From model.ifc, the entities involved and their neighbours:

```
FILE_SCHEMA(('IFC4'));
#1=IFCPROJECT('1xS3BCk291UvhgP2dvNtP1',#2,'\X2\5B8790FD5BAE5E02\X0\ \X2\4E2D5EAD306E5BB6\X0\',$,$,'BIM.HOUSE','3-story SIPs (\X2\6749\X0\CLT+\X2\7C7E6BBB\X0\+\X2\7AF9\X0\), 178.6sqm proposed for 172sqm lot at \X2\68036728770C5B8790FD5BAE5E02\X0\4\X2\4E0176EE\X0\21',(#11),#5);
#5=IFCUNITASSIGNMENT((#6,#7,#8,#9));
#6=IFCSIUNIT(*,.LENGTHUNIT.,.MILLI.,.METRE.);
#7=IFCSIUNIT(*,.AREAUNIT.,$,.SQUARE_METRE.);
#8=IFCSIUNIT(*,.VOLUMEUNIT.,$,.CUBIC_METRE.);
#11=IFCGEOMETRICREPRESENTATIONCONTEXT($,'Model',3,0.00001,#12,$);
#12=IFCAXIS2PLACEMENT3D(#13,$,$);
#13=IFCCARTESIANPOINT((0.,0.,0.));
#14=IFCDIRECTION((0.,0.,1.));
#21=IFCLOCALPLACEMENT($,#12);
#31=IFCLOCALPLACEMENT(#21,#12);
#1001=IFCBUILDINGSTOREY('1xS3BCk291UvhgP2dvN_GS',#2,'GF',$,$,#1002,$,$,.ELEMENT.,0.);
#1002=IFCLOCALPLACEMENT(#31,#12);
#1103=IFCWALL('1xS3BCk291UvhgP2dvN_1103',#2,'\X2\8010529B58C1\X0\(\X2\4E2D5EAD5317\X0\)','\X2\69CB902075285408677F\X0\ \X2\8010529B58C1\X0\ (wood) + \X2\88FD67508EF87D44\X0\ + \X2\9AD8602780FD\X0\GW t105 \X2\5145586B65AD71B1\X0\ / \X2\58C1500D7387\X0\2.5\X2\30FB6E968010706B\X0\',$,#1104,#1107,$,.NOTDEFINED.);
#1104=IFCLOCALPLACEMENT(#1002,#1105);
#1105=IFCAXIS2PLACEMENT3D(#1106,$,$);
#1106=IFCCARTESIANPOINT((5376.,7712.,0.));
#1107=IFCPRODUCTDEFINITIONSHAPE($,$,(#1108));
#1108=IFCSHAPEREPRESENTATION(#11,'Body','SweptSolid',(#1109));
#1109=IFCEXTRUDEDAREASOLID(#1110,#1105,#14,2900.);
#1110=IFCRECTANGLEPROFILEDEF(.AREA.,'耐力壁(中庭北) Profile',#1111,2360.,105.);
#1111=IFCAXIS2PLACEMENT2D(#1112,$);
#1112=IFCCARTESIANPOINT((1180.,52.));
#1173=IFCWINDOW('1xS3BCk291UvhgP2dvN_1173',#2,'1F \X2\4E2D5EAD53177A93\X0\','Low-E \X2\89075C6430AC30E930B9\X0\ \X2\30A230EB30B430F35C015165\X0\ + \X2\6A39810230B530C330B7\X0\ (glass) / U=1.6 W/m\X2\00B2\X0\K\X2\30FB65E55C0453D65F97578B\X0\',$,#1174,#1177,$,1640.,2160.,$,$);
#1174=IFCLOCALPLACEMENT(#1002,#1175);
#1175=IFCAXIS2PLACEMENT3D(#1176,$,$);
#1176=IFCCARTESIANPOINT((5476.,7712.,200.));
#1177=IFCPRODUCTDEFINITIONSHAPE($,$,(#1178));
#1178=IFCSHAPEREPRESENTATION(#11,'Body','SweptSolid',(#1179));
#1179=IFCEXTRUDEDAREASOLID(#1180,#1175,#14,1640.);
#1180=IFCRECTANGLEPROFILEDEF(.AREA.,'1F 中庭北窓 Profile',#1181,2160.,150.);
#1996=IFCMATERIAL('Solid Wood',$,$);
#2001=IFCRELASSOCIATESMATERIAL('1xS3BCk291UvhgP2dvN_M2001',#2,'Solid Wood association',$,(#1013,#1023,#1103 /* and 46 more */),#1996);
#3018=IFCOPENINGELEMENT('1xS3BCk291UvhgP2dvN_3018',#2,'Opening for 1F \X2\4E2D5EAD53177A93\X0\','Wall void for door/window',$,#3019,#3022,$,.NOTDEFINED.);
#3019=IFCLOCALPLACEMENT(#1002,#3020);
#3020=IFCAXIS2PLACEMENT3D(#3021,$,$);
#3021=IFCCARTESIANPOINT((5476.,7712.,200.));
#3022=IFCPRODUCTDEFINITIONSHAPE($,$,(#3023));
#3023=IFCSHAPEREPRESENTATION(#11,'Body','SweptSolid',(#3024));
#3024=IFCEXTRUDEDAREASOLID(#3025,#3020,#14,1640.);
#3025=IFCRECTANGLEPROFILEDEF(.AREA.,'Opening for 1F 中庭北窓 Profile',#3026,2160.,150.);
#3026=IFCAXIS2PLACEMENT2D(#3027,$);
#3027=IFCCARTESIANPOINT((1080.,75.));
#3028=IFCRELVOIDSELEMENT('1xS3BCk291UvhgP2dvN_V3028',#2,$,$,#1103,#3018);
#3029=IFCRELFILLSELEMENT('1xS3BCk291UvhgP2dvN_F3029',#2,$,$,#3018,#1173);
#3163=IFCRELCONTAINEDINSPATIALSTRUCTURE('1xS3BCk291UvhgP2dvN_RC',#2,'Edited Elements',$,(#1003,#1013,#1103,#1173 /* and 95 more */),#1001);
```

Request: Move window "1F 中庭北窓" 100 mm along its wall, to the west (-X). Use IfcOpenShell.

```python
import ifcopenshell
import ifcopenshell.api.geometry
import ifcopenshell.util.placement
import ifcopenshell.util.unit

model = ifcopenshell.open("model.ifc")
unit_scale = ifcopenshell.util.unit.calculate_unit_scale(model)

window = model.by_guid("1xS3BCk291UvhgP2dvN_1173")
opening = window.FillsVoids[0].RelatingOpeningElement
wall = opening.VoidsElements[0].RelatingBuildingElement

wall_matrix = ifcopenshell.util.placement.get_local_placement(wall.ObjectPlacement)
shift = wall_matrix[:3, 0] * -0.1 / unit_scale
before = ifcopenshell.util.placement.get_local_placement(window.ObjectPlacement)[:3, 3].copy()

# The window is not placed relative to its opening, so move both.
for product in (opening, window):
    matrix = ifcopenshell.util.placement.get_local_placement(product.ObjectPlacement)
    matrix[:3, 3] += shift
    ifcopenshell.api.geometry.edit_object_placement(model, product=product, matrix=matrix, is_si=False)

after = ifcopenshell.util.placement.get_local_placement(window.ObjectPlacement)[:3, 3]
print("window moved by", (after - before).round(3) + 0.0)

model.write("model_edited.ifc")
```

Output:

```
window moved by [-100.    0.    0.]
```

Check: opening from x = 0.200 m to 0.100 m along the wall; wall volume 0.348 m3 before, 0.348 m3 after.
